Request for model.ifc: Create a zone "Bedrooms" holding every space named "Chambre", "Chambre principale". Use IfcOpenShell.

First a look at what the model holds.

```python
import ifcopenshell

model = ifcopenshell.open("model.ifc")
print(model.schema)
seen = {}
for space in model.by_type("IfcSpace"):
    seen[space.LongName] = seen.get(space.LongName, 0) + 1
for name, count in sorted(seen.items(), key=str):
    print(count, "x", name)
print("zones:", [z.Name for z in model.by_type("IfcZone")][:20])
```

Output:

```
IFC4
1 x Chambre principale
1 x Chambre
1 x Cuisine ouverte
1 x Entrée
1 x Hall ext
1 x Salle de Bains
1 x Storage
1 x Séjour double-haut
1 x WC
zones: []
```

```python
import ifcopenshell
import ifcopenshell.api.group
import ifcopenshell.api.root

model = ifcopenshell.open("model.ifc")

names = {"Chambre", "Chambre principale"}
spaces = [s for s in model.by_type("IfcSpace") if s.LongName in names]

zone = ifcopenshell.api.root.create_entity(model, ifc_class="IfcZone", name="Bedrooms")
ifcopenshell.api.group.assign_group(model, products=spaces, group=zone)
print(len(spaces), "spaces in", zone.Name)

model.write("model-out.ifc")
```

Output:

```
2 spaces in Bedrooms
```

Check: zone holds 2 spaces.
